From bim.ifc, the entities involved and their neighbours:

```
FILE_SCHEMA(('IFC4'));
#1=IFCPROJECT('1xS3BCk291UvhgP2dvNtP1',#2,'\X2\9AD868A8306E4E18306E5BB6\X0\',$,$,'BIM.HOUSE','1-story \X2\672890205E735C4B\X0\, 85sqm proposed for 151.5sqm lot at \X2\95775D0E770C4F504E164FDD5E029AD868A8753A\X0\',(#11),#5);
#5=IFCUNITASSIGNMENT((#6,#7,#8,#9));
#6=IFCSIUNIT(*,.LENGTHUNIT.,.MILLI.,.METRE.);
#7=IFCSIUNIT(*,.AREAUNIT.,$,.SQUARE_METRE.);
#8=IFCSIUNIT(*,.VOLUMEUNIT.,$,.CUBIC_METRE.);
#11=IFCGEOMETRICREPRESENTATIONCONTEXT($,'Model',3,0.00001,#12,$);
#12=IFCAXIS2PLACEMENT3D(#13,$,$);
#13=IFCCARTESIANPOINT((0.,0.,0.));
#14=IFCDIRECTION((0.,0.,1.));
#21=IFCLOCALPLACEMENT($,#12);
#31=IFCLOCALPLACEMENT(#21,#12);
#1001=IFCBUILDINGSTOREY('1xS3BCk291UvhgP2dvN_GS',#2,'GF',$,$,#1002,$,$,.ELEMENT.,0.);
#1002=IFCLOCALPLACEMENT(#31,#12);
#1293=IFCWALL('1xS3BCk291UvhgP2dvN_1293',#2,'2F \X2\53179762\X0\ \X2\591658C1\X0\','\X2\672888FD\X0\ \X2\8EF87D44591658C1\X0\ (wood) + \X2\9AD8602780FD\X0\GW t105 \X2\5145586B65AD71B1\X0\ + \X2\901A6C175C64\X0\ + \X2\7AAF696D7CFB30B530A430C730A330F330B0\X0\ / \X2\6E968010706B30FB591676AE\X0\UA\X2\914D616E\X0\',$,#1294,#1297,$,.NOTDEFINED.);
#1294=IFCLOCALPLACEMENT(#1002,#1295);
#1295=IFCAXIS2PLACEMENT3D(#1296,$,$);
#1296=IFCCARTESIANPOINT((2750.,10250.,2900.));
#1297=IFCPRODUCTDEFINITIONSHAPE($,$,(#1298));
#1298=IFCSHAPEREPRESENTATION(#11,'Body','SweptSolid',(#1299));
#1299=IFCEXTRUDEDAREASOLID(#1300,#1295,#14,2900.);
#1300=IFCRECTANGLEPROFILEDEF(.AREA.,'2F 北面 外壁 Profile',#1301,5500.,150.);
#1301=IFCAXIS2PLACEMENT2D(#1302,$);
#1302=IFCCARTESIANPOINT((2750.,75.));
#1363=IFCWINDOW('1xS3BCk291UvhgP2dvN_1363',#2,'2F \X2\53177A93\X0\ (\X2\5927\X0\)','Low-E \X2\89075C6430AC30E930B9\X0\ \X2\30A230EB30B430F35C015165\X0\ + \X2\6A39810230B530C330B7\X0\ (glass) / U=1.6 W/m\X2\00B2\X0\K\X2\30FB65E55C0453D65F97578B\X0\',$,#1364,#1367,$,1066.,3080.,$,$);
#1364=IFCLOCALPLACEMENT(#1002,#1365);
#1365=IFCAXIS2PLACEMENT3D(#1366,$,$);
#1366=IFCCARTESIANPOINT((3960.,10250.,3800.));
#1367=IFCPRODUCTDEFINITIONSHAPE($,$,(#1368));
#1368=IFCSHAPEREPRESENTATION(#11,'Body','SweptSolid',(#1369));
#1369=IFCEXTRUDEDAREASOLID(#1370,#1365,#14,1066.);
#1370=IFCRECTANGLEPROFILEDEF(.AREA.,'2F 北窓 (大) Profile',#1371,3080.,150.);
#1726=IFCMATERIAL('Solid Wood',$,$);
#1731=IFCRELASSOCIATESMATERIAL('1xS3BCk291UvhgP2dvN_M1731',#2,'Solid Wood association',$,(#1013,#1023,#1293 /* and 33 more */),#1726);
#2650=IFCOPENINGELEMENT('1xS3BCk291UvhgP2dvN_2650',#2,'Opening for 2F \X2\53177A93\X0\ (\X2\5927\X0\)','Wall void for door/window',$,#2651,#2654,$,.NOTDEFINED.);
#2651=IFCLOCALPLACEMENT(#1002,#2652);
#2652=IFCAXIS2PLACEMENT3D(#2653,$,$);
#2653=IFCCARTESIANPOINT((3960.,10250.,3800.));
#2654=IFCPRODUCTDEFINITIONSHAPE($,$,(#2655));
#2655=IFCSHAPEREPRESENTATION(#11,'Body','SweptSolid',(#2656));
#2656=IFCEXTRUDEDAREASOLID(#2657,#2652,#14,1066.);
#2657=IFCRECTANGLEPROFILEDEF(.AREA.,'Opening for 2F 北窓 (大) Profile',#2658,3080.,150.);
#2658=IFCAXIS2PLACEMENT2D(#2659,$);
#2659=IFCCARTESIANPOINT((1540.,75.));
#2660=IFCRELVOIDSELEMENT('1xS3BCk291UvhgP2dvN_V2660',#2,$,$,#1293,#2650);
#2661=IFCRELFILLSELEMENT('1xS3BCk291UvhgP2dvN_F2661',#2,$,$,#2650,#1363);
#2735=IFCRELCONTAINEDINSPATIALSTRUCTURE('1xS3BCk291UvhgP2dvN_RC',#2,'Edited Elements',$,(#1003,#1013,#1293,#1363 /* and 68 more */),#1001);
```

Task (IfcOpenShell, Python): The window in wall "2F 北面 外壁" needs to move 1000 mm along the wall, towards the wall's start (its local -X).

```python
import ifcopenshell
import ifcopenshell.api.geometry
import ifcopenshell.util.placement

model = ifcopenshell.open("bim.ifc")

window = model.by_guid("1xS3BCk291UvhgP2dvN_1363")
opening = window.FillsVoids[0].RelatingOpeningElement
wall = opening.VoidsElements[0].RelatingBuildingElement

wall_matrix = ifcopenshell.util.placement.get_local_placement(wall.ObjectPlacement)
shift = wall_matrix[:3, 0] * -1000.0
before = ifcopenshell.util.placement.get_local_placement(window.ObjectPlacement)[:3, 3].copy()

# The window is not placed relative to its opening, so move both.
for product in (opening, window):
    matrix = ifcopenshell.util.placement.get_local_placement(product.ObjectPlacement)
    matrix[:3, 3] += shift
    ifcopenshell.api.geometry.edit_object_placement(model, product=product, matrix=matrix, is_si=False)

after = ifcopenshell.util.placement.get_local_placement(window.ObjectPlacement)[:3, 3]
print("window moved by", (after - before).round(3) + 0.0)

model.write("bim_rev.ifc")
```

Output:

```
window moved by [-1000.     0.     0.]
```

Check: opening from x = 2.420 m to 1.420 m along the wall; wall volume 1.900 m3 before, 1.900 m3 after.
